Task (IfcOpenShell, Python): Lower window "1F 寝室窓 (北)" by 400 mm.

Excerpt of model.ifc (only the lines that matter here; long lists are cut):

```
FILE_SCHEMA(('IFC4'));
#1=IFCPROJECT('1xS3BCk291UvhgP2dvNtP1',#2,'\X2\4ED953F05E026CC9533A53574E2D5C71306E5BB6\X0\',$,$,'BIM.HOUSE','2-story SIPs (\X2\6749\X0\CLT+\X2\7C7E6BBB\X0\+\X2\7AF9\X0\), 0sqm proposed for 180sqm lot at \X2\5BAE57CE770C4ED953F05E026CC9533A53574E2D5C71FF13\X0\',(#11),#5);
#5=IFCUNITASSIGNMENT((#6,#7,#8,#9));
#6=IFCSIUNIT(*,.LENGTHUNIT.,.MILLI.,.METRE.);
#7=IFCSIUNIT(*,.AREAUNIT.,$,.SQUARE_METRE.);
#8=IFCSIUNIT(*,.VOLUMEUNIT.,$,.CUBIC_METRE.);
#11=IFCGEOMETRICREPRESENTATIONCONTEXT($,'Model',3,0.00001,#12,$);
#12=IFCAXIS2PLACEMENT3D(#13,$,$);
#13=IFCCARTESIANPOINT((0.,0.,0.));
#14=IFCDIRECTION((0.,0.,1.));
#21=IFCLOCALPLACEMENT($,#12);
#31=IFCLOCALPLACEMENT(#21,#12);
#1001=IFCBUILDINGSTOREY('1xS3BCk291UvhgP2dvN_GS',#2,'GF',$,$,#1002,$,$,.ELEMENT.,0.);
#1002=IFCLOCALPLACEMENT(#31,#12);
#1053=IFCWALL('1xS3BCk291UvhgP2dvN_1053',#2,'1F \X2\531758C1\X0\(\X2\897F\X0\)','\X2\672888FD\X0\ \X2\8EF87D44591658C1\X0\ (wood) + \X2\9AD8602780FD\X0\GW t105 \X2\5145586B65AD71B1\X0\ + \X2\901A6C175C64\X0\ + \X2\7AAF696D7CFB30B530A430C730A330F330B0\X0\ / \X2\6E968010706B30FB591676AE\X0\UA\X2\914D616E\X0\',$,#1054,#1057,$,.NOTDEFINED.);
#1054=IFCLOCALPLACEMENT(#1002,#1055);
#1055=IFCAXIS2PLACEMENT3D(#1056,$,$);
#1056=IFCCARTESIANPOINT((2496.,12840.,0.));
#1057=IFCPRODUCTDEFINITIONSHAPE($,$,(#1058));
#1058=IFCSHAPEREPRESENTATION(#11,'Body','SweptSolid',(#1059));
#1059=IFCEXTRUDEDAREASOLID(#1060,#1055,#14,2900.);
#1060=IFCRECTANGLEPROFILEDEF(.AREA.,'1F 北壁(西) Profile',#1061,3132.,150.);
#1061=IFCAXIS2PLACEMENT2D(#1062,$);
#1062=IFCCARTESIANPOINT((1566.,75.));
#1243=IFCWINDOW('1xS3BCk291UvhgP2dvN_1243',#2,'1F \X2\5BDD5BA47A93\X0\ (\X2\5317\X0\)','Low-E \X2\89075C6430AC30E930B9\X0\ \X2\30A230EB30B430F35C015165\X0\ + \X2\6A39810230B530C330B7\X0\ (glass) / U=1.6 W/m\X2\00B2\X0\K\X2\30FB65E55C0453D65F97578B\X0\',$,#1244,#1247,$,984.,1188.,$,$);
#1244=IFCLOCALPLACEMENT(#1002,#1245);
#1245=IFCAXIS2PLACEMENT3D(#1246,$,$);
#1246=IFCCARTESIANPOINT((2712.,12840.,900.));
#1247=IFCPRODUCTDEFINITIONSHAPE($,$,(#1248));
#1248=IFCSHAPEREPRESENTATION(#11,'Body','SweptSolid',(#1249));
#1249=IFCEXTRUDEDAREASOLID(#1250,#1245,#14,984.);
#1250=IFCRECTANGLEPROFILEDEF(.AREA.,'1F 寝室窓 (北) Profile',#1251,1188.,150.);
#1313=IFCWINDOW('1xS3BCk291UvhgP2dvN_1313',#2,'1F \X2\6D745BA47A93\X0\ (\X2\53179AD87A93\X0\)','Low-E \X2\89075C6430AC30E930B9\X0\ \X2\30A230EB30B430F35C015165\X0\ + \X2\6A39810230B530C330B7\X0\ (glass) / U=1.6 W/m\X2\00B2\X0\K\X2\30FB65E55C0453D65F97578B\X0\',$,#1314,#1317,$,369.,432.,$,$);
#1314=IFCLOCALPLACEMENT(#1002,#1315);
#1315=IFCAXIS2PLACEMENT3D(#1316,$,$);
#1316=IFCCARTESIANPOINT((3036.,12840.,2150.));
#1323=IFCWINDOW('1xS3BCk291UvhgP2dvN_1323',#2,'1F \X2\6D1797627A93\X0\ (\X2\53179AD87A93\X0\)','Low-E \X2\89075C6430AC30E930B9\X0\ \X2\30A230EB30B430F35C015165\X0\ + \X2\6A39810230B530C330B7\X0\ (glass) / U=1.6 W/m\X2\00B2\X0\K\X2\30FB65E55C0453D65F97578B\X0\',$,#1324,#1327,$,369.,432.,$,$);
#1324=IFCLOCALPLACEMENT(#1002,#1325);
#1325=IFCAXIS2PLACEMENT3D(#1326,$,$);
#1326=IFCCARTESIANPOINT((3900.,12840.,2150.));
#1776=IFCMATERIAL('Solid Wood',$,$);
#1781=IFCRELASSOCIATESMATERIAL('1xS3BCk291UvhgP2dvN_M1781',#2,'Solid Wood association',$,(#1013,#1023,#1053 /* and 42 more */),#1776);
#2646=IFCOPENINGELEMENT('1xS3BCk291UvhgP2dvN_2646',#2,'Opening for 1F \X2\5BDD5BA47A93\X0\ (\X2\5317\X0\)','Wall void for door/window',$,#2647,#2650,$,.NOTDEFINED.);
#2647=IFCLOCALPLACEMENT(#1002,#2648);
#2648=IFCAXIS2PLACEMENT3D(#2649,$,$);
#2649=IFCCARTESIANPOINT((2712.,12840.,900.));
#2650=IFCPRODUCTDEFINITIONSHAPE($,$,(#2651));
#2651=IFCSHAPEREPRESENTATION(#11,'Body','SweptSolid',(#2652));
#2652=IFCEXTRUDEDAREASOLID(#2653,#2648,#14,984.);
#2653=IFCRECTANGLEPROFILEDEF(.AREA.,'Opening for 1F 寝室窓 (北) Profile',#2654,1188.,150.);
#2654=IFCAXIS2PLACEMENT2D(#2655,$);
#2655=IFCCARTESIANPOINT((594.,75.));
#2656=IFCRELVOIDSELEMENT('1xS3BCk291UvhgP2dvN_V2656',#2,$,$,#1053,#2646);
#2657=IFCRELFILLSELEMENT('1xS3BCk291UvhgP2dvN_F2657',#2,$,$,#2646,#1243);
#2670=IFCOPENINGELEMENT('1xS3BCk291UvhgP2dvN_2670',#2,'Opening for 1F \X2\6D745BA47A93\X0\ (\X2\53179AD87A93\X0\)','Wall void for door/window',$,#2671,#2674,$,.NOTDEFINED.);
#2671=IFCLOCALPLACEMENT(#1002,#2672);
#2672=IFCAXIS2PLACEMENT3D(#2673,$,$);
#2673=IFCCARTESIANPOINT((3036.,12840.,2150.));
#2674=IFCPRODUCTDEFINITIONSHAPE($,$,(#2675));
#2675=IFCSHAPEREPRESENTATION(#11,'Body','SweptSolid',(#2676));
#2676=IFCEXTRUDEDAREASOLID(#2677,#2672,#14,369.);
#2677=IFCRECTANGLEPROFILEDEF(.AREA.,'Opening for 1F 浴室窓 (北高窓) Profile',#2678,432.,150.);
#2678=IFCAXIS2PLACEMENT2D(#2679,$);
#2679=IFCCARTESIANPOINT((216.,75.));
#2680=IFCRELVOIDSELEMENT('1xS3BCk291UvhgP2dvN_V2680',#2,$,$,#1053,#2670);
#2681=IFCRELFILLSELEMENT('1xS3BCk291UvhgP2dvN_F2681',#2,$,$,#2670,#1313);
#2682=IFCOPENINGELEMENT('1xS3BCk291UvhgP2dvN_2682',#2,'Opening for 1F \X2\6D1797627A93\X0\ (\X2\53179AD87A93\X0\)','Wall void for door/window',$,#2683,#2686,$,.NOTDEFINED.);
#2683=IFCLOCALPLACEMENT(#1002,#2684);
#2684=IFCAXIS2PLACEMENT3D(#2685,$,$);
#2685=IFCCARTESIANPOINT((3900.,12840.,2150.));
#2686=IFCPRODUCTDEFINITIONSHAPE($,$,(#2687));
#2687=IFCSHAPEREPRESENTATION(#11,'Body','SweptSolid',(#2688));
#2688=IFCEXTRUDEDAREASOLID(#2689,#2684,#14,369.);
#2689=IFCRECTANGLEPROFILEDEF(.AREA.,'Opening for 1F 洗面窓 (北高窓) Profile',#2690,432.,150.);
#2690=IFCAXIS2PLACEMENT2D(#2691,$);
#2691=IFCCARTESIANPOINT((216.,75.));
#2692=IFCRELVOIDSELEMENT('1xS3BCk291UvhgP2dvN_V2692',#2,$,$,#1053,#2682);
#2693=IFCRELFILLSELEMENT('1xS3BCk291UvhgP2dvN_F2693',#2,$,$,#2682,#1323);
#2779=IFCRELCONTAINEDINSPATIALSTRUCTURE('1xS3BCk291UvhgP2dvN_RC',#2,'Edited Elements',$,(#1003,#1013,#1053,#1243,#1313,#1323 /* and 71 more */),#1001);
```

```python
import numpy as np
import ifcopenshell
import ifcopenshell.api.geometry
import ifcopenshell.util.placement
import ifcopenshell.util.unit

model = ifcopenshell.open("model.ifc")
unit_scale = ifcopenshell.util.unit.calculate_unit_scale(model)

window = model.by_id(1243)
opening = window.FillsVoids[0].RelatingOpeningElement
dz = -400.0

shift = np.array([0.0, 0.0, dz])
# The window is not placed relative to its opening, so move both.
for product in (opening, window):
    matrix = ifcopenshell.util.placement.get_local_placement(product.ObjectPlacement)
    matrix[:3, 3] += shift
    ifcopenshell.api.geometry.edit_object_placement(model, product=product, matrix=matrix, is_si=False)

print(f"moved by {dz * unit_scale:+.3f} m")

model.write("model_rev.ifc")
```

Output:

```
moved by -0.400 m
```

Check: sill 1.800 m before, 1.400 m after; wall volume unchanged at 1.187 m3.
